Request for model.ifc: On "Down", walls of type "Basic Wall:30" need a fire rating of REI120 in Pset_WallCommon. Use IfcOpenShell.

First a look at what the model holds.

```python
import ifcopenshell
import ifcopenshell.util.element

model = ifcopenshell.open("model.ifc")
print(model.schema)
storey = next(s for s in model.by_type("IfcBuildingStorey") if s.Name == "Down")
walls = [e for e in ifcopenshell.util.element.get_decomposition(storey) if e.is_a("IfcWall")]
seen = {}
for e in walls:
    element_type = ifcopenshell.util.element.get_type(e)
    key = (element_type.Name if element_type != e and element_type else None, ifcopenshell.util.element.get_pset(e, "Pset_WallCommon", "FireRating"))
    seen[key] = seen.get(key, 0) + 1
for (name, value), count in sorted(seen.items(), key=str):
    print(count, "x", name, "|", value)
```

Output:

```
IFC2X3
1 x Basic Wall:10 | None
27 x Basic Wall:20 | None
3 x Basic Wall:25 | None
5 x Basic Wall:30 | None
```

```python
import ifcopenshell
import ifcopenshell.api.pset
import ifcopenshell.util.element

model = ifcopenshell.open("model.ifc")

storey = next(s for s in model.by_type("IfcBuildingStorey") if s.Name == "Down")
walls = [e for e in ifcopenshell.util.element.get_decomposition(storey) if e.is_a("IfcWall")]

count = 0
for e in walls:
    element_type = ifcopenshell.util.element.get_type(e)
    if element_type in (None, e) or element_type.Name != "Basic Wall:30":
        continue
    # add_pset returns the element's existing set when there is one.
    pset = ifcopenshell.api.pset.add_pset(model, product=e, name="Pset_WallCommon")
    ifcopenshell.api.pset.edit_pset(model, pset=pset, properties={"FireRating": "REI120"})
    count += 1

print(count, "walls updated")

model.write("model_rev.ifc")
```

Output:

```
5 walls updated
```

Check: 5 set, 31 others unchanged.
